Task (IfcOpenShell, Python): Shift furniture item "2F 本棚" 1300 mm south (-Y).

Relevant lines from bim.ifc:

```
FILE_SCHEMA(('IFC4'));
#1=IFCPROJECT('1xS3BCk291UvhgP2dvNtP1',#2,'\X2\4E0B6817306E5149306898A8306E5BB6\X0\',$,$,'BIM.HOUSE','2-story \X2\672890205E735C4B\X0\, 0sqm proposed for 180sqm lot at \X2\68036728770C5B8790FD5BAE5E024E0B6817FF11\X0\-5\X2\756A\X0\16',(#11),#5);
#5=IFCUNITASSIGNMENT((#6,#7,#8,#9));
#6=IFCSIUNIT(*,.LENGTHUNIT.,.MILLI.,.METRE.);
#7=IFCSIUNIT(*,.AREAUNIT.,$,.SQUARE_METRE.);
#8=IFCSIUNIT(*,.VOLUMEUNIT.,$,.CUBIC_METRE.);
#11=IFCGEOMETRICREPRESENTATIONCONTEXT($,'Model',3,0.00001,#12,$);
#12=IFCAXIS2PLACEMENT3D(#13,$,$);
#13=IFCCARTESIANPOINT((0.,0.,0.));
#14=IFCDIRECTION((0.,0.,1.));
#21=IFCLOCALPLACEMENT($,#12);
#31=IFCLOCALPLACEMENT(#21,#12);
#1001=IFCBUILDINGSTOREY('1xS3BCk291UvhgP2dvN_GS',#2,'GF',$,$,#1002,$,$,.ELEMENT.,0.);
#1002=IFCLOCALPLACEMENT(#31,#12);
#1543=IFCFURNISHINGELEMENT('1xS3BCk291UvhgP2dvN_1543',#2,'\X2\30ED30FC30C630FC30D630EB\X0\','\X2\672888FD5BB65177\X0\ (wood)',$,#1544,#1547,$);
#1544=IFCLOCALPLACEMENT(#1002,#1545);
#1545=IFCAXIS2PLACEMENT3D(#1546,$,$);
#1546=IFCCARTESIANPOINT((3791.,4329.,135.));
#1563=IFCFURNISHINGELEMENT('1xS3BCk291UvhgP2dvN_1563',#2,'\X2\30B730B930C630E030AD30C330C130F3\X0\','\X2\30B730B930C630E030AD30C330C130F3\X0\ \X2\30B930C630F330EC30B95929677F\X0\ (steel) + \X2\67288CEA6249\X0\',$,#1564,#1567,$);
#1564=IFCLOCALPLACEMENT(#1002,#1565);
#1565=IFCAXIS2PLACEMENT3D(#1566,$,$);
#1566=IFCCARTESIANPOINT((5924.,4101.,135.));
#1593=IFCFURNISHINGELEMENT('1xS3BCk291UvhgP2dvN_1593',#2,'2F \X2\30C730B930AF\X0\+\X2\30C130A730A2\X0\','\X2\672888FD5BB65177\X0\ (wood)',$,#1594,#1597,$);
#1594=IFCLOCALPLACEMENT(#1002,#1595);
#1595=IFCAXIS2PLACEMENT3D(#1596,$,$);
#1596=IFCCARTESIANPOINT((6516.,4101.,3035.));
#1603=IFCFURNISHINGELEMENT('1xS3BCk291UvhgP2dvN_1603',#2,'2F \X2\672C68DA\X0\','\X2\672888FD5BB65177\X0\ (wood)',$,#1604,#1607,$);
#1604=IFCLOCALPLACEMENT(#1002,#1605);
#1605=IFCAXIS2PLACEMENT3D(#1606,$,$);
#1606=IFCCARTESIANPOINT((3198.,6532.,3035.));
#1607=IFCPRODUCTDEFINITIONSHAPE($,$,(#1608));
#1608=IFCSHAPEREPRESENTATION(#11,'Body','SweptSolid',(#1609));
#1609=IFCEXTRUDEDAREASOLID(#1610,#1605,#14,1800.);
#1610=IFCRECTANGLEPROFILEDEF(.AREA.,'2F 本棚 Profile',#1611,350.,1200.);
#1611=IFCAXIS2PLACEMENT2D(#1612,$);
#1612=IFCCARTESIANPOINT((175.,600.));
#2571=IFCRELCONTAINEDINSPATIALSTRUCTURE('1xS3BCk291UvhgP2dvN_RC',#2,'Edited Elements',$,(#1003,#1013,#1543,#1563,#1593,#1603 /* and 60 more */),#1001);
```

```python
import ifcopenshell
import ifcopenshell.api.geometry
import ifcopenshell.util.placement

model = ifcopenshell.open("bim.ifc")

item = model.by_id(1603)
matrix = ifcopenshell.util.placement.get_local_placement(item.ObjectPlacement)
matrix[1, 3] -= 1300.0
ifcopenshell.api.geometry.edit_object_placement(model, product=item, matrix=matrix, is_si=False)

print(ifcopenshell.util.placement.get_local_placement(item.ObjectPlacement).round(3) + 0.0)

model.write("bim_updated.ifc")
```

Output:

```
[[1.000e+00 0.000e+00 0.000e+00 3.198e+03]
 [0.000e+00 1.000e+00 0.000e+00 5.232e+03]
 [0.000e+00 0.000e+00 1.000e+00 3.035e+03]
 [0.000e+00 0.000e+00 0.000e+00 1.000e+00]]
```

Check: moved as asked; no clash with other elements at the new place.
